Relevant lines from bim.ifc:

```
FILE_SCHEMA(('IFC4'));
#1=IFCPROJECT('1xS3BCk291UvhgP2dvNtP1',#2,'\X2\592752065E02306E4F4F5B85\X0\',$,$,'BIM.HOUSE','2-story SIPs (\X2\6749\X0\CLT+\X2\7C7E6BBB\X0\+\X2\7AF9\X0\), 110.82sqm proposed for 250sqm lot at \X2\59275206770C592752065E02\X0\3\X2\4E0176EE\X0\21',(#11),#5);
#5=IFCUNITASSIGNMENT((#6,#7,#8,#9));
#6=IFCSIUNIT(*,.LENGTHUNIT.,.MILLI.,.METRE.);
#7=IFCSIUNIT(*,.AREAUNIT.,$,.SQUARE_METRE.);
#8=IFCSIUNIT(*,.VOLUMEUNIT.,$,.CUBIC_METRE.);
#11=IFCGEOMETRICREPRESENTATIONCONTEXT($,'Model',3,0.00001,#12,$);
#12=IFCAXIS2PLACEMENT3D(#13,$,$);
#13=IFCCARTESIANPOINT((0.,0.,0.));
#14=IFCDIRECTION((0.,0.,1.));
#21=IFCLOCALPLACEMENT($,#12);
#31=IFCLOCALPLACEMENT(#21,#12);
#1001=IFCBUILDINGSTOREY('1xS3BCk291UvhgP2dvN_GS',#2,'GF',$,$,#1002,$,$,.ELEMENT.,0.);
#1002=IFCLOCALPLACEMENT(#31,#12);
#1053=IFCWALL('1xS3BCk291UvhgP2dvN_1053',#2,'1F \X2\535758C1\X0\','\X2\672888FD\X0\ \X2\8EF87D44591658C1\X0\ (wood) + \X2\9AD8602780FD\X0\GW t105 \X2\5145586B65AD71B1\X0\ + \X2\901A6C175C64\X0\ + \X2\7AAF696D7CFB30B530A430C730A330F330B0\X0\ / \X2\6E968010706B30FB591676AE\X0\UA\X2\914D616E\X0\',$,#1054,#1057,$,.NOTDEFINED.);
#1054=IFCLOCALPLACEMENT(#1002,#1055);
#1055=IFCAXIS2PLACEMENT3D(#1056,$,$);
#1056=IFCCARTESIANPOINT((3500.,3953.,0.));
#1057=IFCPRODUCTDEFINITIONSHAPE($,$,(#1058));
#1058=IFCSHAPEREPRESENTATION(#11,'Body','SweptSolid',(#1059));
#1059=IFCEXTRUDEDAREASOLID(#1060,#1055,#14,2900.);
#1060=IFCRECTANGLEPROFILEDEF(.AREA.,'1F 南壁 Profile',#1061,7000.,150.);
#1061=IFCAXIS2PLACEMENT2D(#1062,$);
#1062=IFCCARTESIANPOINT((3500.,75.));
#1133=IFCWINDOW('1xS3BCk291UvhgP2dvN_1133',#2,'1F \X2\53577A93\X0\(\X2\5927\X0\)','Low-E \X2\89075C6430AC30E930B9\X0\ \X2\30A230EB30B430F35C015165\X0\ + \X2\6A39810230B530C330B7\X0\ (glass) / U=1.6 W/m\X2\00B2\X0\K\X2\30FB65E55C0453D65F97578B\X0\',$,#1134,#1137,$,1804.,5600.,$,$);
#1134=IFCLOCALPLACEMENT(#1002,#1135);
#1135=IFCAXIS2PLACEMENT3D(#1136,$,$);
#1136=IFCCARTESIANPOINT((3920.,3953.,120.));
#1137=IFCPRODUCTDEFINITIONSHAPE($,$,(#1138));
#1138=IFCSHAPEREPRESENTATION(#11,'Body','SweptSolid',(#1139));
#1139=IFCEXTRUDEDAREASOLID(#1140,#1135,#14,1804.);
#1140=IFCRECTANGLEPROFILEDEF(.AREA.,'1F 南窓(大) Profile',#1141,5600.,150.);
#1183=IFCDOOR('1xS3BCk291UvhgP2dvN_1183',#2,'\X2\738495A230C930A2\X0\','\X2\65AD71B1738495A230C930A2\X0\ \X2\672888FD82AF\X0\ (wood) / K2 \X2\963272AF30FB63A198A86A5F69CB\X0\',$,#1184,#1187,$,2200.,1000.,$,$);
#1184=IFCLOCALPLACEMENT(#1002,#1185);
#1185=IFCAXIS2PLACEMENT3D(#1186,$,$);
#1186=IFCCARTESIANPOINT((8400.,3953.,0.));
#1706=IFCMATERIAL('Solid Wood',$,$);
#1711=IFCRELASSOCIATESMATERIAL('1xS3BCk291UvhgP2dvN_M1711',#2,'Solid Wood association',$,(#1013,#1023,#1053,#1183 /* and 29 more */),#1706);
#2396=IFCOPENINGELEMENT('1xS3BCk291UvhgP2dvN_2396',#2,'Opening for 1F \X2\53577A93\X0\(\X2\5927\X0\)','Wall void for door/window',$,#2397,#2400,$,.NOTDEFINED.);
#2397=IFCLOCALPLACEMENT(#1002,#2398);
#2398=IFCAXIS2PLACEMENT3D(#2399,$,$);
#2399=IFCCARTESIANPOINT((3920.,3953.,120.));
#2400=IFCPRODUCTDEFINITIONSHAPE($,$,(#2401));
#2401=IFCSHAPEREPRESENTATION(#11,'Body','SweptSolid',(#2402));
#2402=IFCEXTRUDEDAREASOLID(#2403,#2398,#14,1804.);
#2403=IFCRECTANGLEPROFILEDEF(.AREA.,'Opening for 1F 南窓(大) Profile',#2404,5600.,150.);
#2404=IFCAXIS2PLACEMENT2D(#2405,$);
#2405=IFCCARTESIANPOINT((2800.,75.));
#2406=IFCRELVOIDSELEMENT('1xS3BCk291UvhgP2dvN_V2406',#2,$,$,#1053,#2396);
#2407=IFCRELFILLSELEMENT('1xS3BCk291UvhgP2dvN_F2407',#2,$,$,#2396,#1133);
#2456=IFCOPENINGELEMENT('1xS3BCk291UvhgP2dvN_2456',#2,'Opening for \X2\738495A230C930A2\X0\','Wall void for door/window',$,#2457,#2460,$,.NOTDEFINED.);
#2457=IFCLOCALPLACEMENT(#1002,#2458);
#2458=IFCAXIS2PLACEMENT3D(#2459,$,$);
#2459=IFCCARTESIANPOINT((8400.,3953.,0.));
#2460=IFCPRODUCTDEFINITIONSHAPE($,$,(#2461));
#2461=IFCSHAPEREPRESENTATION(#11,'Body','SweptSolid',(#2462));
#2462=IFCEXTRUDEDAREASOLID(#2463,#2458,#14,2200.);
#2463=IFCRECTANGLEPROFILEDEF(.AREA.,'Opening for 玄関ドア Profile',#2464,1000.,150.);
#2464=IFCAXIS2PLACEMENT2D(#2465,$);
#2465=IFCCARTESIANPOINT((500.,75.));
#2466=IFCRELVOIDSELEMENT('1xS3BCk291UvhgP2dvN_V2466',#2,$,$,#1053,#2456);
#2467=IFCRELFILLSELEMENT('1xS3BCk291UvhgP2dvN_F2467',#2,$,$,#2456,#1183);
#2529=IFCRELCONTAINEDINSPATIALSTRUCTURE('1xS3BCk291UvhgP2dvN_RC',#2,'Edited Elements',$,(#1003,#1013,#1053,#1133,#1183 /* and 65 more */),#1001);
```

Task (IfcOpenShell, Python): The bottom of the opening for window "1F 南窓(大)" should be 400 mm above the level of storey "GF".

```python
import numpy as np
import ifcopenshell
import ifcopenshell.api.geometry
import ifcopenshell.geom
import ifcopenshell.util.element
import ifcopenshell.util.placement
import ifcopenshell.util.shape
import ifcopenshell.util.unit

model = ifcopenshell.open("bim.ifc")
unit_scale = ifcopenshell.util.unit.calculate_unit_scale(model)

window = model.by_guid("1xS3BCk291UvhgP2dvN_1133")
opening = window.FillsVoids[0].RelatingOpeningElement
storey = ifcopenshell.util.element.get_container(window, ifc_class="IfcBuildingStorey")
level = ifcopenshell.util.placement.get_local_placement(storey.ObjectPlacement)[2, 3]

# The opening's origin need not be at the sill, so measure its lowest point.
shape = ifcopenshell.geom.create_shape(ifcopenshell.geom.settings(), opening)
bottom = ifcopenshell.util.shape.get_shape_bottom_elevation(shape, shape.geometry) / unit_scale
dz = level + 0.4 / unit_scale - bottom

shift = np.array([0.0, 0.0, dz])
# The window is not placed relative to its opening, so move both.
for product in (opening, window):
    matrix = ifcopenshell.util.placement.get_local_placement(product.ObjectPlacement)
    matrix[:3, 3] += shift
    ifcopenshell.api.geometry.edit_object_placement(model, product=product, matrix=matrix, is_si=False)

print(f"moved by {dz * unit_scale:+.3f} m")

model.write("bim_v2.ifc")
```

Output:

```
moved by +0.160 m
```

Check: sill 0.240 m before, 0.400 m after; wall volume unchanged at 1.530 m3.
